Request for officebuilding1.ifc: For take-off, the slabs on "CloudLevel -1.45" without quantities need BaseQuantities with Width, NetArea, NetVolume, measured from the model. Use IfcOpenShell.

First a look at what the model holds.

```python
import ifcopenshell
import ifcopenshell.util.element
import ifcopenshell.util.unit

model = ifcopenshell.open("officebuilding1.ifc")
print(model.schema)
for unit_type in ("LENGTHUNIT", "AREAUNIT", "VOLUMEUNIT"):
    print(unit_type, ifcopenshell.util.unit.calculate_unit_scale(model, unit_type))
storey = next(s for s in model.by_type("IfcBuildingStorey") if s.Name == "CloudLevel -1.45")
slabs = [e for e in ifcopenshell.util.element.get_decomposition(storey) if e.is_a("IfcSlab")]
for e in sorted(slabs, key=lambda e: e.id()):
    print(e.id(), e.is_a(), e.Name, list(ifcopenshell.util.element.get_psets(e, qtos_only=True)), sep=" | ")
```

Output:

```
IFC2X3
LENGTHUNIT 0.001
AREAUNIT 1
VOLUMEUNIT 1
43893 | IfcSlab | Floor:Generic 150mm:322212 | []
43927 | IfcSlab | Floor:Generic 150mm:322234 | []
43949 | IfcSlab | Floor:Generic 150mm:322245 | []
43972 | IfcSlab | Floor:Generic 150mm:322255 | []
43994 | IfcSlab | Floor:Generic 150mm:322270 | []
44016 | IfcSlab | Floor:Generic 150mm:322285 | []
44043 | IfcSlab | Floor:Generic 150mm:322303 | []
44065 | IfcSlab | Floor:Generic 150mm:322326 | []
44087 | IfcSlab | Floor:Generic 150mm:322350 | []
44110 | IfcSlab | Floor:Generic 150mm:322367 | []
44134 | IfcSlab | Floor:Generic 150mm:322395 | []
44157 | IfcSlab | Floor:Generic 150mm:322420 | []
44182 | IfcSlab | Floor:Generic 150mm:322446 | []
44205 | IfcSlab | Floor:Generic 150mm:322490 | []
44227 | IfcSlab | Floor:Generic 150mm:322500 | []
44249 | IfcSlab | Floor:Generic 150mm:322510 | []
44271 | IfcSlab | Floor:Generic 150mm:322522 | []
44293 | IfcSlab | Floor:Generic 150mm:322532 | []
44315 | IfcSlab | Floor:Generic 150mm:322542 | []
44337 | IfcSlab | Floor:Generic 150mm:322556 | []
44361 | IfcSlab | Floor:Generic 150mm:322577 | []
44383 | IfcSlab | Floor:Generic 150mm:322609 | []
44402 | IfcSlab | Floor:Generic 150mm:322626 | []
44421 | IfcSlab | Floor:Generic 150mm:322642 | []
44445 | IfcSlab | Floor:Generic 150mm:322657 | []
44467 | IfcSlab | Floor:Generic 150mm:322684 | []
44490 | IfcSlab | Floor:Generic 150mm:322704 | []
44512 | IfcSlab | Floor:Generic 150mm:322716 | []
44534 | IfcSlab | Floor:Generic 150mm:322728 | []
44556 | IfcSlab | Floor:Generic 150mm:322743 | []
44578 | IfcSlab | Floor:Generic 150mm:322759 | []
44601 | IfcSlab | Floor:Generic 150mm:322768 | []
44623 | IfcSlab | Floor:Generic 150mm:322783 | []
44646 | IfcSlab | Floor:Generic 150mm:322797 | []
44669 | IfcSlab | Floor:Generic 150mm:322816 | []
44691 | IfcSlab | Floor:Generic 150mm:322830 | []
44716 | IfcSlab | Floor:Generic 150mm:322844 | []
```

```python
import ifcopenshell
import ifcopenshell.api.pset
import ifcopenshell.geom
import ifcopenshell.util.element
import ifcopenshell.util.shape
import ifcopenshell.util.unit

model = ifcopenshell.open("officebuilding1.ifc")
unit_scale = ifcopenshell.util.unit.calculate_unit_scale(model)
area_scale = ifcopenshell.util.unit.calculate_unit_scale(model, "AREAUNIT")
volume_scale = ifcopenshell.util.unit.calculate_unit_scale(model, "VOLUMEUNIT")
settings = ifcopenshell.geom.settings()

storey = next(s for s in model.by_type("IfcBuildingStorey") if s.Name == "CloudLevel -1.45")
slabs = [e for e in ifcopenshell.util.element.get_decomposition(storey) if e.is_a("IfcSlab")]

for e in sorted(slabs, key=lambda e: e.id()):
    if ifcopenshell.util.element.get_psets(e, qtos_only=True, should_inherit=False):
        continue
    # Geometry comes back in metres, in the element's own axes.
    shape = ifcopenshell.geom.create_shape(settings, e)
    values = {
        "Width": ifcopenshell.util.shape.get_z(shape.geometry) / unit_scale,
        "NetArea": ifcopenshell.util.shape.get_footprint_area(shape.geometry) / area_scale,
        "NetVolume": ifcopenshell.util.shape.get_volume(shape.geometry) / volume_scale,
    }
    qto = ifcopenshell.api.pset.add_qto(model, product=e, name="BaseQuantities")
    ifcopenshell.api.pset.edit_qto(model, qto=qto, properties=values)
    print(e.id(), {k: round(v, 3) for k, v in values.items()})

model.write("officebuilding1_v2.ifc")
```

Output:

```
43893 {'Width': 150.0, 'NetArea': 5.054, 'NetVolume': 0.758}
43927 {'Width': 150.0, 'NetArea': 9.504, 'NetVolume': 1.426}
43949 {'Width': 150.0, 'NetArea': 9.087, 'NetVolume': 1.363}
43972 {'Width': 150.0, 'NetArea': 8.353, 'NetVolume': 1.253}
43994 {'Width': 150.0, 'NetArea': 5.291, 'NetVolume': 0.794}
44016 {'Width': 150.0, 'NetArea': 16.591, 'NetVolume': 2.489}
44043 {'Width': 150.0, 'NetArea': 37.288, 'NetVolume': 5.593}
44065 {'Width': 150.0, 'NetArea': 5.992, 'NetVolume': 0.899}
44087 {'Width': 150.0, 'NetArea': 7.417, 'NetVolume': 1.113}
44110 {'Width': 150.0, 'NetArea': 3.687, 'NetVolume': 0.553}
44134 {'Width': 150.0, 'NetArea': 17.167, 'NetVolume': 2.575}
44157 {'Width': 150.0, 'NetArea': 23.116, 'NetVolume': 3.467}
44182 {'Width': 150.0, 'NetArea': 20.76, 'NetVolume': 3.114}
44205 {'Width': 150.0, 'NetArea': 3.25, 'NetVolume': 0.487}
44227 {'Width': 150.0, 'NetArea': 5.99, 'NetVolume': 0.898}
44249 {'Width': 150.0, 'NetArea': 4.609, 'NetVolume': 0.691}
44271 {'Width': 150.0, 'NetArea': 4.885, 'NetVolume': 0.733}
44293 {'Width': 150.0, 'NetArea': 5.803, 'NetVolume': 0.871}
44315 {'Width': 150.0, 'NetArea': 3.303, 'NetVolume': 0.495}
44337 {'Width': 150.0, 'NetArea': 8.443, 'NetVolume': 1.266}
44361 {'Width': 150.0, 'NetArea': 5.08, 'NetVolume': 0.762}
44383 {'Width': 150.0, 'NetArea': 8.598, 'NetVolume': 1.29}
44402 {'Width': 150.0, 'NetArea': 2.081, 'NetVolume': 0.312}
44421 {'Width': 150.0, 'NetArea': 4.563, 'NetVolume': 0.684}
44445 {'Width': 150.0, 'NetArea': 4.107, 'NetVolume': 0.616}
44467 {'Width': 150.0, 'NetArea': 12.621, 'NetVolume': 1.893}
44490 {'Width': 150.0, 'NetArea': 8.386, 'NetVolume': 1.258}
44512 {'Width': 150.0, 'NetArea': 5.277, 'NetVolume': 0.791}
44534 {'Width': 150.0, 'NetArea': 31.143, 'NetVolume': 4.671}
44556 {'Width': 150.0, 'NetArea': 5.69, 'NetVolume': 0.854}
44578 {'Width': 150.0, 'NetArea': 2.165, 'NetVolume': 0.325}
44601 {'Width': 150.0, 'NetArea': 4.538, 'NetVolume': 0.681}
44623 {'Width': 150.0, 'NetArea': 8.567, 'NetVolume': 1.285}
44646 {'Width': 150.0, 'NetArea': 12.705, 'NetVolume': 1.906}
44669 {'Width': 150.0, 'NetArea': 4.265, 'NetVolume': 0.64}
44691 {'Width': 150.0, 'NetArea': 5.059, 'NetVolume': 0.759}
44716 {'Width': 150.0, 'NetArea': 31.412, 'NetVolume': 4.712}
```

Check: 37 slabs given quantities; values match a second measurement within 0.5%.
